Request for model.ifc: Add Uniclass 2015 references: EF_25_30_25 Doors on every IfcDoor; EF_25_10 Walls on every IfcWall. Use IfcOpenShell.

First a look at what the model holds.

```python
import ifcopenshell

model = ifcopenshell.open("model.ifc")
print(model.schema)
print("classifications:", [c.Name for c in model.by_type("IfcClassification")])
for ifc_class in ("IfcDoor", "IfcRoof", "IfcStair", "IfcWall", "IfcWindow"):
    print(ifc_class, len(model.by_type(ifc_class)))
```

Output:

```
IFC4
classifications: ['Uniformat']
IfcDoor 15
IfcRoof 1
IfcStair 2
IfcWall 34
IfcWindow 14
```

```python
import ifcopenshell
import ifcopenshell.api.classification

model = ifcopenshell.open("model.ifc")

system = ifcopenshell.api.classification.add_classification(model, classification="Uniclass 2015")

codes = {
    "IfcDoor": ("EF_25_30_25", "Doors"),
    "IfcWall": ("EF_25_10", "Walls"),
}
for ifc_class, (code, name) in codes.items():
    products = model.by_type(ifc_class)
    ifcopenshell.api.classification.add_reference(
        model, products=products, classification=system, identification=code, name=name
    )
    print(code, len(products))

model.write("model-out.ifc")
```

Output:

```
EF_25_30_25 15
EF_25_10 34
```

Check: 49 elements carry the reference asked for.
